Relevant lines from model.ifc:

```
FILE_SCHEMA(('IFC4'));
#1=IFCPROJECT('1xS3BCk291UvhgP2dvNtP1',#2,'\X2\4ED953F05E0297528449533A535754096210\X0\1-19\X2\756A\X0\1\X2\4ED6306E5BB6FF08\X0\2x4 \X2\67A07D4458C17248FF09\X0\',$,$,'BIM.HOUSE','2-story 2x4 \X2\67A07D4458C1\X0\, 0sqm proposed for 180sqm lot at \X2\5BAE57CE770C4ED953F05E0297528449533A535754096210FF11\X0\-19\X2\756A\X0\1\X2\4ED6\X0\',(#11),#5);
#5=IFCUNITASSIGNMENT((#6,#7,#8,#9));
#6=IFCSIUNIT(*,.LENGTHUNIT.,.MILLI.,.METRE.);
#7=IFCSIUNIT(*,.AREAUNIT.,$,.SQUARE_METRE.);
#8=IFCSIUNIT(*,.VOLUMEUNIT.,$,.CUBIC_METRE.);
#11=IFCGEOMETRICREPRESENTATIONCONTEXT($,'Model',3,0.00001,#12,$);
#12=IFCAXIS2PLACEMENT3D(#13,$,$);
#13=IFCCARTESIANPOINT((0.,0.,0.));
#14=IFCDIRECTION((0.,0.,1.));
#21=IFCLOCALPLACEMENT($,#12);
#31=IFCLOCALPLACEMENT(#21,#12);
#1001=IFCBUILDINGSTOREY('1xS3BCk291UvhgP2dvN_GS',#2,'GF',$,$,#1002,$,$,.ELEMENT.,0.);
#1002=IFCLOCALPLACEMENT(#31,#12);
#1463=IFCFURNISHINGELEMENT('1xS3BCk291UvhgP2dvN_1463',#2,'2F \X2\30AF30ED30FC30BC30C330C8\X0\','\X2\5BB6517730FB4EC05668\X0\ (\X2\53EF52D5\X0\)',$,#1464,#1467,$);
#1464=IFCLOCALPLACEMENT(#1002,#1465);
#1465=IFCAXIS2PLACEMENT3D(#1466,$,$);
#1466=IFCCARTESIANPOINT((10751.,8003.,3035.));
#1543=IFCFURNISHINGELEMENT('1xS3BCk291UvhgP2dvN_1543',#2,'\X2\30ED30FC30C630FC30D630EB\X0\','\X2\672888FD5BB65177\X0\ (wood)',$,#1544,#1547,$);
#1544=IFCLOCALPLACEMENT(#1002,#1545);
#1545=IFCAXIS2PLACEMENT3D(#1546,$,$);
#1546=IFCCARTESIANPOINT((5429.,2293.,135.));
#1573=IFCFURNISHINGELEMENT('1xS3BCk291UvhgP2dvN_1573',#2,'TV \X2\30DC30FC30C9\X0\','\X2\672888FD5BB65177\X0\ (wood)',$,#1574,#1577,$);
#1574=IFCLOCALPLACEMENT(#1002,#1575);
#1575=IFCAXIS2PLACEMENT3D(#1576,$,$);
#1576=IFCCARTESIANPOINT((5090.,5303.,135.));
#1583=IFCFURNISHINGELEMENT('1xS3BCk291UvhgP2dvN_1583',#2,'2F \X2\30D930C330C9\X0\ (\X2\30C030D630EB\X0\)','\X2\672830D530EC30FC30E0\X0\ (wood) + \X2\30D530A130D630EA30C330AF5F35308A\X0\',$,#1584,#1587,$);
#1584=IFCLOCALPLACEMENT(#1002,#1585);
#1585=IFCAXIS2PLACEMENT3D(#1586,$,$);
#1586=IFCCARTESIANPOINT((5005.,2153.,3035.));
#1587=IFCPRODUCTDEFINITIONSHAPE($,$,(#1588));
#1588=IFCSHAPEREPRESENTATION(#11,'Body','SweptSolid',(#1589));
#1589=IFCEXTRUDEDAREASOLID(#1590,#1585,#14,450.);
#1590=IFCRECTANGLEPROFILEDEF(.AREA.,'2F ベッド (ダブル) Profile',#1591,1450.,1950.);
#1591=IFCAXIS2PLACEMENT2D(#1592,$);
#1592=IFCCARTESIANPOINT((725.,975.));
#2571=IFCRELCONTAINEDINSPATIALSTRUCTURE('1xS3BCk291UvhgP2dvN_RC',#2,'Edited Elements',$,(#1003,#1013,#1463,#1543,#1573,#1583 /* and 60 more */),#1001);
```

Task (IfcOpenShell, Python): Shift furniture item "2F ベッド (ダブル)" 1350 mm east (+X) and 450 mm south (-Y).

```python
import ifcopenshell
import ifcopenshell.api.geometry
import ifcopenshell.util.placement

model = ifcopenshell.open("model.ifc")

item = model.by_guid("1xS3BCk291UvhgP2dvN_1583")
matrix = ifcopenshell.util.placement.get_local_placement(item.ObjectPlacement)
matrix[0, 3] += 1350.0
matrix[1, 3] -= 450.0
ifcopenshell.api.geometry.edit_object_placement(model, product=item, matrix=matrix, is_si=False)

print(ifcopenshell.util.placement.get_local_placement(item.ObjectPlacement).round(3) + 0.0)

model.write("model-out.ifc")
```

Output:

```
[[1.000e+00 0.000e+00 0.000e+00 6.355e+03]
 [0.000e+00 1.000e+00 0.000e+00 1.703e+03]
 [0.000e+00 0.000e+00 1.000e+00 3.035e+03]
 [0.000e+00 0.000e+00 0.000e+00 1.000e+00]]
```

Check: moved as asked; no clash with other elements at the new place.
